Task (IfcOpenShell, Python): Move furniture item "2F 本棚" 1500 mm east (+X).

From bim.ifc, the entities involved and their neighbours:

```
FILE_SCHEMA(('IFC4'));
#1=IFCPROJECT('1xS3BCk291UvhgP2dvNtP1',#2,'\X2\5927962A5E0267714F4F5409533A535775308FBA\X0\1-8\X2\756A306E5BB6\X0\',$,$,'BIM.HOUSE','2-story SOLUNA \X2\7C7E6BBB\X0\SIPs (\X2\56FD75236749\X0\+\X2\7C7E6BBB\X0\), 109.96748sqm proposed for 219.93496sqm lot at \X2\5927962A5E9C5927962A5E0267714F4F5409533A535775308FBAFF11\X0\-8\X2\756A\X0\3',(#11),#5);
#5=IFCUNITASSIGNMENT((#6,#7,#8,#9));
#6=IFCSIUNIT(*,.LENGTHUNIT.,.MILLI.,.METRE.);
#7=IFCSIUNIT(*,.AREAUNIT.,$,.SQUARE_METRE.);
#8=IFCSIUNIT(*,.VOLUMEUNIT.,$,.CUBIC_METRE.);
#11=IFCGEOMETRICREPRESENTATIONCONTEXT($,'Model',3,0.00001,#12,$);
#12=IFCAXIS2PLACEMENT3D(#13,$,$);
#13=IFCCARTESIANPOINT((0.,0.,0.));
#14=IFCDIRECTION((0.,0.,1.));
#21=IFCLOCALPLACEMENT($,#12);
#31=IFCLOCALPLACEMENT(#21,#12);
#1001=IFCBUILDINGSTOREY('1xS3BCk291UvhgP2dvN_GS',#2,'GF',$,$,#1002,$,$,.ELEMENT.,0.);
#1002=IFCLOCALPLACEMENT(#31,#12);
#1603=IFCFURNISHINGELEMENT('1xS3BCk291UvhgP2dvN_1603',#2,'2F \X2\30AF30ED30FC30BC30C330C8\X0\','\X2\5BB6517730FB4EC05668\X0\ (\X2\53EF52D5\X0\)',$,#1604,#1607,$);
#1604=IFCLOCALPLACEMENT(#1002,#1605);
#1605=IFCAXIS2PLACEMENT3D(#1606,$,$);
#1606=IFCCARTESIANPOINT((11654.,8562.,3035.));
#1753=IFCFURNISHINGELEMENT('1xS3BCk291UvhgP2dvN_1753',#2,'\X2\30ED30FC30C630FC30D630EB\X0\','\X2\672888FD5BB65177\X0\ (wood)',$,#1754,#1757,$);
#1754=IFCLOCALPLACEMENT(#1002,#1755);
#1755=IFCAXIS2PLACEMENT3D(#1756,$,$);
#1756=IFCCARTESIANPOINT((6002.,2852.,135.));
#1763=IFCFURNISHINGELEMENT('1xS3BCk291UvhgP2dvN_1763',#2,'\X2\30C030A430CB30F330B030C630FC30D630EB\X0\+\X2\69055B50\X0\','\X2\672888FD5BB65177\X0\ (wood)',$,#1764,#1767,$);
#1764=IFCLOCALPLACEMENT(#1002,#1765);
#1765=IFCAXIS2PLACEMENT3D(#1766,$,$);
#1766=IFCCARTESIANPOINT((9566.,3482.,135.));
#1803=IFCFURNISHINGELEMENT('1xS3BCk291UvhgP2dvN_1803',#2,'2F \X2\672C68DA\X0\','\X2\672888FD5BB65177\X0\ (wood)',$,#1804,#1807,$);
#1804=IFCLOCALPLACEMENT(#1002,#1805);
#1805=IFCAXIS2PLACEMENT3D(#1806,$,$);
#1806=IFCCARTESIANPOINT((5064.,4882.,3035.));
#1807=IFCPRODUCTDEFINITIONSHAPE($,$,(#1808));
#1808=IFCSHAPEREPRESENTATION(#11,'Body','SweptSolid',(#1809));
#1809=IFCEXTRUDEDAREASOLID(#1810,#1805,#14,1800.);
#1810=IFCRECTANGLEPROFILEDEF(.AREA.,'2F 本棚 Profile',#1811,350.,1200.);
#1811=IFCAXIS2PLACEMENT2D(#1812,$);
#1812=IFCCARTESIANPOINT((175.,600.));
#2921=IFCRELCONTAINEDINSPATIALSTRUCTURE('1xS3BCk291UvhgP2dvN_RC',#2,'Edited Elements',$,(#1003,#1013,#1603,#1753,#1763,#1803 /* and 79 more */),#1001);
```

```python
import ifcopenshell
import ifcopenshell.api.geometry
import ifcopenshell.util.placement

model = ifcopenshell.open("bim.ifc")

item = model.by_guid("1xS3BCk291UvhgP2dvN_1803")
matrix = ifcopenshell.util.placement.get_local_placement(item.ObjectPlacement)
matrix[0, 3] += 1500.0
ifcopenshell.api.geometry.edit_object_placement(model, product=item, matrix=matrix, is_si=False)

print(ifcopenshell.util.placement.get_local_placement(item.ObjectPlacement).round(3) + 0.0)

model.write("bim_v2.ifc")
```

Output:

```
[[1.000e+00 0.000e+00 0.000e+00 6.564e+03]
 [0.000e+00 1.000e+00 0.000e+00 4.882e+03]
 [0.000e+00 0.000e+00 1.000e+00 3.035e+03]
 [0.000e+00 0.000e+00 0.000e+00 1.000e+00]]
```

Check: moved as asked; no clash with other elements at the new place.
